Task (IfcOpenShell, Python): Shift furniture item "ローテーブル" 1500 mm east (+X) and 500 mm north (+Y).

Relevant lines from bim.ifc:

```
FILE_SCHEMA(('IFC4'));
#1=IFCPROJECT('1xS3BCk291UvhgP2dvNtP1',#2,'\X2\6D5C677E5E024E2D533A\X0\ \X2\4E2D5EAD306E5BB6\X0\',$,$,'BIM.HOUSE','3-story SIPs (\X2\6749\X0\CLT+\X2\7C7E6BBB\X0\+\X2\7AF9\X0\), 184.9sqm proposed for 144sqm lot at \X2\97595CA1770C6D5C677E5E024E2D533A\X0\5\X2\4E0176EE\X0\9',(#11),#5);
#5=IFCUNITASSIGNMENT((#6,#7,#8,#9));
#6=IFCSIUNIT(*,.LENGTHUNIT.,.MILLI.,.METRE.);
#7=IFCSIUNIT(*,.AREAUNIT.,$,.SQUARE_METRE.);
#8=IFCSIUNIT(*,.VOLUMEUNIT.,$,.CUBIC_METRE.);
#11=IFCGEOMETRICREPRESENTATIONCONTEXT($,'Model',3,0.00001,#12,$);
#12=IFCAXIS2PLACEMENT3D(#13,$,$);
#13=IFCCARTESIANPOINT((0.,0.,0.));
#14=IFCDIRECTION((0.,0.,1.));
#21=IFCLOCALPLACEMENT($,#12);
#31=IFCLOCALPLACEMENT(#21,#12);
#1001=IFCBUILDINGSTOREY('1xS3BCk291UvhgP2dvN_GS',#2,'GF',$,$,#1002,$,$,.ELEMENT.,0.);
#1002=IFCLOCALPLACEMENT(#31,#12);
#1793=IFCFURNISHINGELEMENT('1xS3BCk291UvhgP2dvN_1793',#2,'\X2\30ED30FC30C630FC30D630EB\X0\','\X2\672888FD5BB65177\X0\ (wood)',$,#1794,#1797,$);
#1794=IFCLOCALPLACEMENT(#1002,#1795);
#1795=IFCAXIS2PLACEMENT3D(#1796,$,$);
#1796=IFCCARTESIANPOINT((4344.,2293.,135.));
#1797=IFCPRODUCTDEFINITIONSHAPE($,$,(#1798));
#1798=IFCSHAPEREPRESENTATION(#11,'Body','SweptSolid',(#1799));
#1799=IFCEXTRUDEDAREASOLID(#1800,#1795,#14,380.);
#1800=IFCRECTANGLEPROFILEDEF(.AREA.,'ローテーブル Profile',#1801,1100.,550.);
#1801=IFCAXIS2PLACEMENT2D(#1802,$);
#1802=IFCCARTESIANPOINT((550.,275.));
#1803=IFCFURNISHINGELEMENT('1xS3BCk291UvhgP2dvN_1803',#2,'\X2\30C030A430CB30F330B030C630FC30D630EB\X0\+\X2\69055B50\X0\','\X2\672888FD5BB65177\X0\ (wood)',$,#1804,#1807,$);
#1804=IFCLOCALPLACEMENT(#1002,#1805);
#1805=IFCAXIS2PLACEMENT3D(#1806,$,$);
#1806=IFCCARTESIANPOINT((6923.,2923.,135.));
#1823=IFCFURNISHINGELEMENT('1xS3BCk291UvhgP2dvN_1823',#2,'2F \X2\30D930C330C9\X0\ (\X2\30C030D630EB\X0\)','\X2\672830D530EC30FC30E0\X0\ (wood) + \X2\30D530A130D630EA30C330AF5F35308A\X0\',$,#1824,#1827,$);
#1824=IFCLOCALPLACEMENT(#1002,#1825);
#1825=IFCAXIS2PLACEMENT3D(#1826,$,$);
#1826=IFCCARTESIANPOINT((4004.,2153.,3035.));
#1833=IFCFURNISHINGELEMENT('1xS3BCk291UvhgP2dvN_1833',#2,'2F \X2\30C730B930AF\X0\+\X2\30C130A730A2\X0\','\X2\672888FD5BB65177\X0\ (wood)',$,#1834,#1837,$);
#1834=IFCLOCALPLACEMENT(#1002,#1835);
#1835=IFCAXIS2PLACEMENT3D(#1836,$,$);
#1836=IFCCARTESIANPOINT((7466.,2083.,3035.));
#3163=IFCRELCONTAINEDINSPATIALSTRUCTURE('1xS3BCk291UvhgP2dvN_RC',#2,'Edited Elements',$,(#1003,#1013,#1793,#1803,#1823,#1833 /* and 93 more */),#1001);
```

```python
import ifcopenshell
import ifcopenshell.api.geometry
import ifcopenshell.util.placement

model = ifcopenshell.open("bim.ifc")

item = model.by_guid("1xS3BCk291UvhgP2dvN_1793")
matrix = ifcopenshell.util.placement.get_local_placement(item.ObjectPlacement)
matrix[0, 3] += 1500.0
matrix[1, 3] += 500.0
ifcopenshell.api.geometry.edit_object_placement(model, product=item, matrix=matrix, is_si=False)

print(ifcopenshell.util.placement.get_local_placement(item.ObjectPlacement).round(3) + 0.0)

model.write("bim_edited.ifc")
```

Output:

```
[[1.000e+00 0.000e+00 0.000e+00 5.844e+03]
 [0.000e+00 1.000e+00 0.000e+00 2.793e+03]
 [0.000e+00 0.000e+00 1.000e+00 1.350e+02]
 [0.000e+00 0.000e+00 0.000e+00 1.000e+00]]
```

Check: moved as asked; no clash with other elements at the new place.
